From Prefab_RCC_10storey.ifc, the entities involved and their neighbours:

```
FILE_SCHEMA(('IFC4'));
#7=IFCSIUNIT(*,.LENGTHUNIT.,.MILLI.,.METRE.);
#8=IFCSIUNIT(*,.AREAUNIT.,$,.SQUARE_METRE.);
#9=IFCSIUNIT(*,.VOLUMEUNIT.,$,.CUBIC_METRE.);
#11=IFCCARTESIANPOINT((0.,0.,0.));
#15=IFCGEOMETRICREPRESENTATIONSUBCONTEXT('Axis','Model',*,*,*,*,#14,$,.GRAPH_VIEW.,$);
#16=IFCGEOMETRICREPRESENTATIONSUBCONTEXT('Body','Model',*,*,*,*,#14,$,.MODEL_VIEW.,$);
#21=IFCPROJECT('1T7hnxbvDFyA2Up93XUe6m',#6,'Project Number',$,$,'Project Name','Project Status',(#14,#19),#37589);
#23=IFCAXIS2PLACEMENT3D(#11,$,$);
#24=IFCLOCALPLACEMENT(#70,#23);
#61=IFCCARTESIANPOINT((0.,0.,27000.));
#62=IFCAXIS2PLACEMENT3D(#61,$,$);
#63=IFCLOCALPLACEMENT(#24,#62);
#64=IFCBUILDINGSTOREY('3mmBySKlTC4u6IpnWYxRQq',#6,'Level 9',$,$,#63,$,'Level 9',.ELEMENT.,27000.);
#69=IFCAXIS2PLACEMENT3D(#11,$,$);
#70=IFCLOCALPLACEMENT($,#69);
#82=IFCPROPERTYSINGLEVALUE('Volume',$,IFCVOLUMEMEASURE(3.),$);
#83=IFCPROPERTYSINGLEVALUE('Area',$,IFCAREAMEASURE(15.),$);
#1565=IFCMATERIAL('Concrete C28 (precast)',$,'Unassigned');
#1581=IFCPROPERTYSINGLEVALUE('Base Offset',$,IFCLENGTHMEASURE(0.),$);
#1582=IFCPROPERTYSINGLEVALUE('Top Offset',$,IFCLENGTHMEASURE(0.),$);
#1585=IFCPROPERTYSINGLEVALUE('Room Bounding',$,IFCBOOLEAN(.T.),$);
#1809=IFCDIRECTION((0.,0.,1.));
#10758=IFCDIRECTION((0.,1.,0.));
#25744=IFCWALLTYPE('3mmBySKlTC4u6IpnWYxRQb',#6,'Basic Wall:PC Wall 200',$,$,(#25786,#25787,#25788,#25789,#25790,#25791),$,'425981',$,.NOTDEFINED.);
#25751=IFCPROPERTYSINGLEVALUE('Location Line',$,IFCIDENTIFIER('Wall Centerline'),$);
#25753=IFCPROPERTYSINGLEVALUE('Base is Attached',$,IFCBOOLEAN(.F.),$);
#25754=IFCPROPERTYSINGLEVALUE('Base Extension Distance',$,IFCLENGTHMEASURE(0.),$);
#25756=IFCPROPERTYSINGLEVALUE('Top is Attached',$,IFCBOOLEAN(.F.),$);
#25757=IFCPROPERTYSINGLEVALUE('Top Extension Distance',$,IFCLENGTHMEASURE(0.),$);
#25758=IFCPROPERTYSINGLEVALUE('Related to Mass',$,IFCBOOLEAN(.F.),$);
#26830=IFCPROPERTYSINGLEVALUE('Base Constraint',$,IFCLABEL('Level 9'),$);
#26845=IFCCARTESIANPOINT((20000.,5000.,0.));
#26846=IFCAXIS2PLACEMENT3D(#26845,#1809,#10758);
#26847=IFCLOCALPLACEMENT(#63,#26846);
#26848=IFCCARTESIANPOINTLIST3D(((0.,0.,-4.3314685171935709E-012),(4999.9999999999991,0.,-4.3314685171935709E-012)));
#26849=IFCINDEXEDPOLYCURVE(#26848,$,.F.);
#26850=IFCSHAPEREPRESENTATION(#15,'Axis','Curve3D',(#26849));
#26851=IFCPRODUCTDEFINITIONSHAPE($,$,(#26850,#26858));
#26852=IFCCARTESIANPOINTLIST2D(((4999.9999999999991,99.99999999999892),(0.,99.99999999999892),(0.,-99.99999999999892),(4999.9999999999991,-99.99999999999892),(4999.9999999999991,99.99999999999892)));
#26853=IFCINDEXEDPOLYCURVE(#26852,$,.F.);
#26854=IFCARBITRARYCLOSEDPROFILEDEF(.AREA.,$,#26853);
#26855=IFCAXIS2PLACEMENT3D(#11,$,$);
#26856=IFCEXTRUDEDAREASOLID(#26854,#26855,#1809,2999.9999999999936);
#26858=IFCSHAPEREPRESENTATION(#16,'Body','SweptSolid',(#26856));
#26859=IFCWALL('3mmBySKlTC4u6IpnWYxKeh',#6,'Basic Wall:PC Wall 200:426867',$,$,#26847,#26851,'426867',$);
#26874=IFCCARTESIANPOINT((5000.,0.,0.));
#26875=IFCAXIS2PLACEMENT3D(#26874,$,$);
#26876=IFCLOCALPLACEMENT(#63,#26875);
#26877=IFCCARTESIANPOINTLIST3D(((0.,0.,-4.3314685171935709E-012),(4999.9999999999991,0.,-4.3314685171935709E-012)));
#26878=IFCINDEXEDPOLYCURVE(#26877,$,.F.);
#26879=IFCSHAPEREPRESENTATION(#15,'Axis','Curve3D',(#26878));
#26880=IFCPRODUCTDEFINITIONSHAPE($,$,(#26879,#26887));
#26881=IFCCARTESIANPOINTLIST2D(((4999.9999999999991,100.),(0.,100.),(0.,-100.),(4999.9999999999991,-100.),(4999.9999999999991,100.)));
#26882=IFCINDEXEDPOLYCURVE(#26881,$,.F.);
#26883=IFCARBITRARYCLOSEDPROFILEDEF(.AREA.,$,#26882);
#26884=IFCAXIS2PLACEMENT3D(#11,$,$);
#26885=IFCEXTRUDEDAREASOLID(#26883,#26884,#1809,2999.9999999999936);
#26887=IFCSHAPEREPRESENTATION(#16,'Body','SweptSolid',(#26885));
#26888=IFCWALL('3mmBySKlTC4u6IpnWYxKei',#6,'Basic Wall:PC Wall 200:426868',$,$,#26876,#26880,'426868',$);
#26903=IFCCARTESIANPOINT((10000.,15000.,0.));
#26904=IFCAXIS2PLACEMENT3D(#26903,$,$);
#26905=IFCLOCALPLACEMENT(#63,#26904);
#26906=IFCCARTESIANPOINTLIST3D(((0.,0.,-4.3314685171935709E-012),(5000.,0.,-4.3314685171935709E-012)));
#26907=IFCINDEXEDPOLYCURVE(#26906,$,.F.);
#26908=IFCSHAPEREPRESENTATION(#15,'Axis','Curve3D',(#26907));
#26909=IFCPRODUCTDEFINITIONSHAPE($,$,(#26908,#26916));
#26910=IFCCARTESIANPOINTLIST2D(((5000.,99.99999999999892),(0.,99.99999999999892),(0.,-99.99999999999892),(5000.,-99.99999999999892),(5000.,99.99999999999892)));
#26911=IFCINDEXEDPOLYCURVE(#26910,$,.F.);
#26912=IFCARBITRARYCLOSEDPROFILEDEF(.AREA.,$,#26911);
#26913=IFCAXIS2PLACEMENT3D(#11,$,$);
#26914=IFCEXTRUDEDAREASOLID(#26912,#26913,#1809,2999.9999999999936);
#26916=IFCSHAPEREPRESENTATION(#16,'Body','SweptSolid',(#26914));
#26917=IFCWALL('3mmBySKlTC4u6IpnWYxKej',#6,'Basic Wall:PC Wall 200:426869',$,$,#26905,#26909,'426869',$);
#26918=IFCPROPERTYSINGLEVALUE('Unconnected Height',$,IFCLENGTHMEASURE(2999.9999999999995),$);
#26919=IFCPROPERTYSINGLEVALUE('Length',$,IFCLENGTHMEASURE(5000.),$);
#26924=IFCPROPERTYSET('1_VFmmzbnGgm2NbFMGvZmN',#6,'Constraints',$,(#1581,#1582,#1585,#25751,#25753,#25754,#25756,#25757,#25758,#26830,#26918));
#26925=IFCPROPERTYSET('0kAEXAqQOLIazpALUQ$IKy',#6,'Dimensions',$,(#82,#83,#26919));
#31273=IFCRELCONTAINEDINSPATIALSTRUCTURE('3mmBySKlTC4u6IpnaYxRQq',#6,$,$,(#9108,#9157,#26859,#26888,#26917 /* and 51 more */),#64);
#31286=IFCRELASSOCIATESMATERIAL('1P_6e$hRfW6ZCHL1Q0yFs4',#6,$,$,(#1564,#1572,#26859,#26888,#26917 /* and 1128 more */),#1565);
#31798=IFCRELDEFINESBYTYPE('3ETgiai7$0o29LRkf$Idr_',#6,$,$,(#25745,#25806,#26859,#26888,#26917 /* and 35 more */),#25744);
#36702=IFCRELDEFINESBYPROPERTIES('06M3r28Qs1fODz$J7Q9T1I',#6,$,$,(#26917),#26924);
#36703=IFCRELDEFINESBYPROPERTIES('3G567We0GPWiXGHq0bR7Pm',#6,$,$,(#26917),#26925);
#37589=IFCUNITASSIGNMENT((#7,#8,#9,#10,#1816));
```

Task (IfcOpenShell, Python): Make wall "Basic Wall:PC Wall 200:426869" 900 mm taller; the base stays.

```python
import ifcopenshell
import ifcopenshell.api.pset
import ifcopenshell.geom
import ifcopenshell.util.element
import ifcopenshell.util.representation
import ifcopenshell.util.shape
import ifcopenshell.util.unit

model = ifcopenshell.open("Prefab_RCC_10storey.ifc")
area_scale = ifcopenshell.util.unit.calculate_unit_scale(model, "AREAUNIT")
volume_scale = ifcopenshell.util.unit.calculate_unit_scale(model, "VOLUMEUNIT")
settings = ifcopenshell.geom.settings()


def volume(element):
    """Net volume in cubic metres, openings subtracted."""
    shape = ifcopenshell.geom.create_shape(settings, element)
    return ifcopenshell.util.shape.get_volume(shape.geometry)


wall = model.by_guid("3mmBySKlTC4u6IpnWYxKej")
before = volume(wall)

body = ifcopenshell.util.representation.get_representation(wall, "Model", "Body")
solid = body.Items[0]
old_height = solid.Depth
solid.Depth += 900.0
after = volume(wall)
thickness = 0.2  # wall thickness in metres

# Update the stored height, areas and volumes.
pset = model.by_id(ifcopenshell.util.element.get_pset(wall, "Constraints", should_inherit=False)["id"])
ifcopenshell.api.pset.edit_pset(model, pset=pset, properties={
    "Unconnected Height": model.create_entity("IfcLengthMeasure", solid.Depth),
})
pset = model.by_id(ifcopenshell.util.element.get_pset(wall, "Dimensions", should_inherit=False)["id"])
ifcopenshell.api.pset.edit_pset(model, pset=pset, properties={
    "Volume": model.create_entity("IfcVolumeMeasure", after / volume_scale),
    "Area": model.create_entity("IfcAreaMeasure", after / thickness / area_scale),
})

print(f"height {old_height:g} -> {solid.Depth:g}, volume {before:.3f} -> {after:.3f} m3")

model.write("Prefab_RCC_10storey_v2.ifc")
```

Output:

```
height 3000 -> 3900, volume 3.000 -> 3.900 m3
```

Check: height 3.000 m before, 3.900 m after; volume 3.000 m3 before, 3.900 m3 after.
